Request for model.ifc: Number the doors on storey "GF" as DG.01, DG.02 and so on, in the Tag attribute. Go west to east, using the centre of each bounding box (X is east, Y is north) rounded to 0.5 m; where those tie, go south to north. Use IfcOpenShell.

First a look at what the model holds.

```python
import ifcopenshell
import ifcopenshell.util.element
import ifcopenshell.util.placement

model = ifcopenshell.open("model.ifc")
print(model.schema)
storey = next(s for s in model.by_type("IfcBuildingStorey") if s.Name == "GF")
doors = [e for e in ifcopenshell.util.element.get_decomposition(storey) if e.is_a("IfcDoor")]
for e in sorted(doors, key=lambda e: e.id()):
    origin = ifcopenshell.util.placement.get_local_placement(e.ObjectPlacement)[:3, 3]
    print(e.id(), e.Tag, e.Name, origin.round(2) + 0.0, sep=" | ")
```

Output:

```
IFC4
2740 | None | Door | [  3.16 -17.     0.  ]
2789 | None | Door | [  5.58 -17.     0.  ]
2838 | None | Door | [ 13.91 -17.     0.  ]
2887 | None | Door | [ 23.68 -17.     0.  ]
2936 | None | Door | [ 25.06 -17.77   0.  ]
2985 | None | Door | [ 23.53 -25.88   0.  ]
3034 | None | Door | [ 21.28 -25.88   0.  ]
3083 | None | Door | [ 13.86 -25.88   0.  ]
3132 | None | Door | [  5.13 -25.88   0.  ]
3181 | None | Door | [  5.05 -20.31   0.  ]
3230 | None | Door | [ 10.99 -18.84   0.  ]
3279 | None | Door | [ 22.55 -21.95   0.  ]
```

```python
import ifcopenshell
import ifcopenshell.geom
import ifcopenshell.util.element
import ifcopenshell.util.shape

model = ifcopenshell.open("model.ifc")
settings = ifcopenshell.geom.settings()
settings.set("use-world-coords", True)


def centre(element):
    shape = ifcopenshell.geom.create_shape(settings, element)
    return ifcopenshell.util.shape.get_bbox_centroid(shape.geometry)


storey = next(s for s in model.by_type("IfcBuildingStorey") if s.Name == "GF")
doors = [e for e in ifcopenshell.util.element.get_decomposition(storey) if e.is_a("IfcDoor")]

# Insertion points can sit at a corner or the storey origin, so sort by the geometry (in metres).
centres = {e: centre(e) for e in doors}
doors.sort(key=lambda e: (round(centres[e][0] / 0.5), centres[e][1]))

for i, e in enumerate(doors, start=1):
    number = f"DG.{i:02d}"
    e.Tag = number
    print(e.id(), number)

model.write("model_edited.ifc")
```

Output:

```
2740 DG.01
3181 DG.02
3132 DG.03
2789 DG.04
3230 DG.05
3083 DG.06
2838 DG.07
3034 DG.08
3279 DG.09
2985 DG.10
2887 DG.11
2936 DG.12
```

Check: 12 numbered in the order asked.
